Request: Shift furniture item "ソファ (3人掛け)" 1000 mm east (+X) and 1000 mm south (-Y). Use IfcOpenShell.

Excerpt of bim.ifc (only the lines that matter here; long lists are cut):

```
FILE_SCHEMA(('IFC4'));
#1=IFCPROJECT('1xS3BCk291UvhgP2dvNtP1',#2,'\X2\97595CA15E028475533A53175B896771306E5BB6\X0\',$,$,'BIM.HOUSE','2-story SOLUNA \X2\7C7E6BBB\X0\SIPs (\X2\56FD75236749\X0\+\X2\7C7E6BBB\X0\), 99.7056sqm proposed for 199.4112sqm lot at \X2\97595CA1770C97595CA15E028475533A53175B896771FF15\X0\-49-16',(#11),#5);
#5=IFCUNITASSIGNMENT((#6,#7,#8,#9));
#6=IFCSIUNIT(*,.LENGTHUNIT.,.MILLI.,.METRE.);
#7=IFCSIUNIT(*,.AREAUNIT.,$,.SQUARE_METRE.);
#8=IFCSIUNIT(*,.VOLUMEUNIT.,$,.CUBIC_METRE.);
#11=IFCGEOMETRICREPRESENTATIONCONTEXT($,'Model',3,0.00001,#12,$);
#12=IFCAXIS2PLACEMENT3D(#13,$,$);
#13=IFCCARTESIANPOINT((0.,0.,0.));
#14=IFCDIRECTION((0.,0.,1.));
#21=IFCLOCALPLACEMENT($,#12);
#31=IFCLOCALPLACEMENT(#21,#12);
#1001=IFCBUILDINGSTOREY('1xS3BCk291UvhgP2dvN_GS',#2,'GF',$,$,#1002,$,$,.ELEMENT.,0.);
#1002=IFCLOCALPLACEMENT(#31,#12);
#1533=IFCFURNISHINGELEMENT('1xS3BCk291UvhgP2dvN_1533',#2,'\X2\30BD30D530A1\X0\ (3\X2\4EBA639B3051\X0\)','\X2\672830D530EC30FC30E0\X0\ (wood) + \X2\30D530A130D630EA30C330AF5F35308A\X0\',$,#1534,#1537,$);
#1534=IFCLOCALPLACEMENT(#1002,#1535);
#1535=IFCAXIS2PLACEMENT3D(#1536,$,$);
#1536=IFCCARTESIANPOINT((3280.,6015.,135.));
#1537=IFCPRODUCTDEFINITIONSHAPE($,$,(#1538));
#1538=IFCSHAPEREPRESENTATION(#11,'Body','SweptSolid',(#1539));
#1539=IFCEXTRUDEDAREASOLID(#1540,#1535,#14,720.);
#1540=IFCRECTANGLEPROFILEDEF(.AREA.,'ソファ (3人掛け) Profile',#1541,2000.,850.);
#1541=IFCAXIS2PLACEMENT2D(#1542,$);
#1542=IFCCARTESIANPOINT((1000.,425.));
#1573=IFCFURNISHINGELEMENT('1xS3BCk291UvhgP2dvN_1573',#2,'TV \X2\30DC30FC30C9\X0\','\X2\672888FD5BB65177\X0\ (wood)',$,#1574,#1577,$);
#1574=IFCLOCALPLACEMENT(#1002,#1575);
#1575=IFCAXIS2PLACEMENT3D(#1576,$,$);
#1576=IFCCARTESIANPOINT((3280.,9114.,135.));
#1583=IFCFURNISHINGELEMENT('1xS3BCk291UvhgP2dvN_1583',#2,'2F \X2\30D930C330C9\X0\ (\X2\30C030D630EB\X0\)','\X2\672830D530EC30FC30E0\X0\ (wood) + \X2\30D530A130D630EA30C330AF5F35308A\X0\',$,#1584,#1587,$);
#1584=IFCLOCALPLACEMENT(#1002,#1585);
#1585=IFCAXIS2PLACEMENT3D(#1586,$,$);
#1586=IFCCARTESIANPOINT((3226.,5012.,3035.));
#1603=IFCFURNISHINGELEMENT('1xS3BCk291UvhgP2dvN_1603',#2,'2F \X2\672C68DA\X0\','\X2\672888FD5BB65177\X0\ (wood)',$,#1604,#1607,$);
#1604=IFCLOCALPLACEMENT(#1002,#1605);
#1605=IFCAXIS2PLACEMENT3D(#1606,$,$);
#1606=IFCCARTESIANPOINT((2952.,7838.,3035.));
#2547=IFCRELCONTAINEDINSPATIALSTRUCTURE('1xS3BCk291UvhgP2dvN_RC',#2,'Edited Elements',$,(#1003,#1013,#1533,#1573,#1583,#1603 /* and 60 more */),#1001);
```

```python
import ifcopenshell
import ifcopenshell.api.geometry
import ifcopenshell.util.placement

model = ifcopenshell.open("bim.ifc")

item = model.by_guid("1xS3BCk291UvhgP2dvN_1533")
matrix = ifcopenshell.util.placement.get_local_placement(item.ObjectPlacement)
matrix[0, 3] += 1000.0
matrix[1, 3] -= 1000.0
ifcopenshell.api.geometry.edit_object_placement(model, product=item, matrix=matrix, is_si=False)

print(ifcopenshell.util.placement.get_local_placement(item.ObjectPlacement).round(3) + 0.0)

model.write("bim_edited.ifc")
```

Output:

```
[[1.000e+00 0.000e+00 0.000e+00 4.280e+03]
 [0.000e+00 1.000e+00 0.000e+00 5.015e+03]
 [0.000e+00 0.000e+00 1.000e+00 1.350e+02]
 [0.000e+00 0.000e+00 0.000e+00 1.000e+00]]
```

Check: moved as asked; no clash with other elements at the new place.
